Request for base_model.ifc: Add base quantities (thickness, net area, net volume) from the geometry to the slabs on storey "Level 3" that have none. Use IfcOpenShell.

First a look at what the model holds.

```python
import ifcopenshell
import ifcopenshell.util.element
import ifcopenshell.util.unit

model = ifcopenshell.open("base_model.ifc")
print(model.schema)
for unit_type in ("LENGTHUNIT", "AREAUNIT", "VOLUMEUNIT"):
    print(unit_type, ifcopenshell.util.unit.calculate_unit_scale(model, unit_type))
storey = next(s for s in model.by_type("IfcBuildingStorey") if s.Name == "Level 3")
slabs = [e for e in ifcopenshell.util.element.get_decomposition(storey) if e.is_a("IfcSlab")]
for e in sorted(slabs, key=lambda e: e.id()):
    print(e.id(), e.is_a(), e.Name, list(ifcopenshell.util.element.get_psets(e, qtos_only=True)), sep=" | ")
```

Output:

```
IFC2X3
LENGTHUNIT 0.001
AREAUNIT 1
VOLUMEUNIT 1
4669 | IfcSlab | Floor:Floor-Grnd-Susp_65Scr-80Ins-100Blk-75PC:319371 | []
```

```python
import ifcopenshell
import ifcopenshell.api.pset
import ifcopenshell.geom
import ifcopenshell.util.element
import ifcopenshell.util.shape
import ifcopenshell.util.unit

model = ifcopenshell.open("base_model.ifc")
unit_scale = ifcopenshell.util.unit.calculate_unit_scale(model)
area_scale = ifcopenshell.util.unit.calculate_unit_scale(model, "AREAUNIT")
volume_scale = ifcopenshell.util.unit.calculate_unit_scale(model, "VOLUMEUNIT")
settings = ifcopenshell.geom.settings()

storey = next(s for s in model.by_type("IfcBuildingStorey") if s.Name == "Level 3")
slabs = [e for e in ifcopenshell.util.element.get_decomposition(storey) if e.is_a("IfcSlab")]

for e in sorted(slabs, key=lambda e: e.id()):
    if ifcopenshell.util.element.get_psets(e, qtos_only=True, should_inherit=False):
        continue
    # Geometry comes back in metres, in the element's own axes.
    shape = ifcopenshell.geom.create_shape(settings, e)
    values = {
        "Width": ifcopenshell.util.shape.get_z(shape.geometry) / unit_scale,
        "NetArea": ifcopenshell.util.shape.get_footprint_area(shape.geometry) / area_scale,
        "NetVolume": ifcopenshell.util.shape.get_volume(shape.geometry) / volume_scale,
    }
    qto = ifcopenshell.api.pset.add_qto(model, product=e, name="BaseQuantities")
    ifcopenshell.api.pset.edit_qto(model, qto=qto, properties=values)
    print(e.id(), {k: round(v, 3) for k, v in values.items()})

model.write("base_model_edited.ifc")
```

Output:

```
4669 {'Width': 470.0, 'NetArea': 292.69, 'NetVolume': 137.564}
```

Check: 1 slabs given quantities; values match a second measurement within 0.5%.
